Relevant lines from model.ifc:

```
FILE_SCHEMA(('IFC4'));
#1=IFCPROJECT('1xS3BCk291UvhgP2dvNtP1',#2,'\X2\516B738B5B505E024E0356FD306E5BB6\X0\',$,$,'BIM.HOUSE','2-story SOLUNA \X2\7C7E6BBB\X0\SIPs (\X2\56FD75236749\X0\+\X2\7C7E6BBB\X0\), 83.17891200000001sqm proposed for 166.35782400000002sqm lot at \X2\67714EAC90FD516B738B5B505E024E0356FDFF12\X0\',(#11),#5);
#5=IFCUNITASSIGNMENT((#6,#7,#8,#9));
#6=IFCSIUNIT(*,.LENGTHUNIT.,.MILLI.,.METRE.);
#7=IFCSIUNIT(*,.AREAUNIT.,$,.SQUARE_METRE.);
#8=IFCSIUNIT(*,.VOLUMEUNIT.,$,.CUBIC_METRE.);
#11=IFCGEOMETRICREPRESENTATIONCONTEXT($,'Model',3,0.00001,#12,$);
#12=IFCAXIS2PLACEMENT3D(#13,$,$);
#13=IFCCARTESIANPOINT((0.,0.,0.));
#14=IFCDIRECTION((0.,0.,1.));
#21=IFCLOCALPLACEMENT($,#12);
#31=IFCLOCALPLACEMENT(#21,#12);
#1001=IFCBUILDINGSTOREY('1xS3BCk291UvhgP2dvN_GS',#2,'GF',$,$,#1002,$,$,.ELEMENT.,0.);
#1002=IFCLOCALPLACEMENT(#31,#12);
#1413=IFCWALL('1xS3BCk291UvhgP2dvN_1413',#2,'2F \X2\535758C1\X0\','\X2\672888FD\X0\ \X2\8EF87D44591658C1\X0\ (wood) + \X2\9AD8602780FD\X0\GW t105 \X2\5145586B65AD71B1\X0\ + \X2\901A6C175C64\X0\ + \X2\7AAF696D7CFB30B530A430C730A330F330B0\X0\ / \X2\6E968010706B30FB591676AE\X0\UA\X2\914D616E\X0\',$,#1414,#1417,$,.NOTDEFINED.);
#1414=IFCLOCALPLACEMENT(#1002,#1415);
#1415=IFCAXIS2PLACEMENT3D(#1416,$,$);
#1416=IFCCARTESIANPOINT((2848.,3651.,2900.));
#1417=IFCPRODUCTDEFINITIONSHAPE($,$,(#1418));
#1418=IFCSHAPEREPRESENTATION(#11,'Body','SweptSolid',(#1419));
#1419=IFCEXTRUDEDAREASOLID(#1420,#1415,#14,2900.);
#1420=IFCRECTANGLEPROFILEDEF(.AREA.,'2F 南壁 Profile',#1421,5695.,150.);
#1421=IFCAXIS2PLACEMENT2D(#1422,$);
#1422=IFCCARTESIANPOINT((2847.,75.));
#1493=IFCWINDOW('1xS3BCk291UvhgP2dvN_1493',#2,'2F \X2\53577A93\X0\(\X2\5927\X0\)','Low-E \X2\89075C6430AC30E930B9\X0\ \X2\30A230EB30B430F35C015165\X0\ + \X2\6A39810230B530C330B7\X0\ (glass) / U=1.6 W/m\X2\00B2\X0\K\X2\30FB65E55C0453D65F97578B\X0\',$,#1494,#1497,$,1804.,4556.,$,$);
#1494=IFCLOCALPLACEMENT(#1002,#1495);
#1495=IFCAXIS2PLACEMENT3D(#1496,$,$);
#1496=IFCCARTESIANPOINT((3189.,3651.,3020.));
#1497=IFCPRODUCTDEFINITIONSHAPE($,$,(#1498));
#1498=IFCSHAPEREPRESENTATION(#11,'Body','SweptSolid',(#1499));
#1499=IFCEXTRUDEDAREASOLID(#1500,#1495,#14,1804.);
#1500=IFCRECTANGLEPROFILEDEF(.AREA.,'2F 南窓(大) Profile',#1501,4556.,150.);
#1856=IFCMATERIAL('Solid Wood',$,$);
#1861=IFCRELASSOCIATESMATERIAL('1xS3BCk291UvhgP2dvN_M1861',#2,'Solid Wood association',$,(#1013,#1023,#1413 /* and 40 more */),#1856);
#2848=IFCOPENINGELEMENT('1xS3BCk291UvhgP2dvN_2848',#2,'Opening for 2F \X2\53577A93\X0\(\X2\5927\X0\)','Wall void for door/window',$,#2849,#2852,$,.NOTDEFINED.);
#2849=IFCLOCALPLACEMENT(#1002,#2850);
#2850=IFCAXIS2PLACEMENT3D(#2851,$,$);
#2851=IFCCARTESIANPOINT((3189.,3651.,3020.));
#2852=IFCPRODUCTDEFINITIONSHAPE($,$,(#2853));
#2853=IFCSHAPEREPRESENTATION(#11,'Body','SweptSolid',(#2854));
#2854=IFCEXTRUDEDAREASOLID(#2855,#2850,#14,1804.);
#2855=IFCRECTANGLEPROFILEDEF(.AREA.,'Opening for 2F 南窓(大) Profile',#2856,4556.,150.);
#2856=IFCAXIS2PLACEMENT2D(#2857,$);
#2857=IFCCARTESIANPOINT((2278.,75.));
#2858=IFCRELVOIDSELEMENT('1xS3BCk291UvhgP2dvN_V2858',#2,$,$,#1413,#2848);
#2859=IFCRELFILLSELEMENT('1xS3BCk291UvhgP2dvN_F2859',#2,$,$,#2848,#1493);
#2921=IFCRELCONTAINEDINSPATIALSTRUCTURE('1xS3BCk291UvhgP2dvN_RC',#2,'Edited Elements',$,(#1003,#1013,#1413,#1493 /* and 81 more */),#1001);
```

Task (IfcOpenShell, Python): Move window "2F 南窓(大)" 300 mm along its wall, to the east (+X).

```python
import ifcopenshell
import ifcopenshell.api.geometry
import ifcopenshell.util.placement

model = ifcopenshell.open("model.ifc")

window = model.by_id(1493)
opening = window.FillsVoids[0].RelatingOpeningElement
wall = opening.VoidsElements[0].RelatingBuildingElement

wall_matrix = ifcopenshell.util.placement.get_local_placement(wall.ObjectPlacement)
shift = wall_matrix[:3, 0] * 300.0
before = ifcopenshell.util.placement.get_local_placement(window.ObjectPlacement)[:3, 3].copy()

# The window is not placed relative to its opening, so move both.
for product in (opening, window):
    matrix = ifcopenshell.util.placement.get_local_placement(product.ObjectPlacement)
    matrix[:3, 3] += shift
    ifcopenshell.api.geometry.edit_object_placement(model, product=product, matrix=matrix, is_si=False)

after = ifcopenshell.util.placement.get_local_placement(window.ObjectPlacement)[:3, 3]
print("window moved by", (after - before).round(3) + 0.0)

model.write("model_v2.ifc")
```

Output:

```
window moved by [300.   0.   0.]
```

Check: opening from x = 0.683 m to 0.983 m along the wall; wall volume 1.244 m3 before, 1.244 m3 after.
